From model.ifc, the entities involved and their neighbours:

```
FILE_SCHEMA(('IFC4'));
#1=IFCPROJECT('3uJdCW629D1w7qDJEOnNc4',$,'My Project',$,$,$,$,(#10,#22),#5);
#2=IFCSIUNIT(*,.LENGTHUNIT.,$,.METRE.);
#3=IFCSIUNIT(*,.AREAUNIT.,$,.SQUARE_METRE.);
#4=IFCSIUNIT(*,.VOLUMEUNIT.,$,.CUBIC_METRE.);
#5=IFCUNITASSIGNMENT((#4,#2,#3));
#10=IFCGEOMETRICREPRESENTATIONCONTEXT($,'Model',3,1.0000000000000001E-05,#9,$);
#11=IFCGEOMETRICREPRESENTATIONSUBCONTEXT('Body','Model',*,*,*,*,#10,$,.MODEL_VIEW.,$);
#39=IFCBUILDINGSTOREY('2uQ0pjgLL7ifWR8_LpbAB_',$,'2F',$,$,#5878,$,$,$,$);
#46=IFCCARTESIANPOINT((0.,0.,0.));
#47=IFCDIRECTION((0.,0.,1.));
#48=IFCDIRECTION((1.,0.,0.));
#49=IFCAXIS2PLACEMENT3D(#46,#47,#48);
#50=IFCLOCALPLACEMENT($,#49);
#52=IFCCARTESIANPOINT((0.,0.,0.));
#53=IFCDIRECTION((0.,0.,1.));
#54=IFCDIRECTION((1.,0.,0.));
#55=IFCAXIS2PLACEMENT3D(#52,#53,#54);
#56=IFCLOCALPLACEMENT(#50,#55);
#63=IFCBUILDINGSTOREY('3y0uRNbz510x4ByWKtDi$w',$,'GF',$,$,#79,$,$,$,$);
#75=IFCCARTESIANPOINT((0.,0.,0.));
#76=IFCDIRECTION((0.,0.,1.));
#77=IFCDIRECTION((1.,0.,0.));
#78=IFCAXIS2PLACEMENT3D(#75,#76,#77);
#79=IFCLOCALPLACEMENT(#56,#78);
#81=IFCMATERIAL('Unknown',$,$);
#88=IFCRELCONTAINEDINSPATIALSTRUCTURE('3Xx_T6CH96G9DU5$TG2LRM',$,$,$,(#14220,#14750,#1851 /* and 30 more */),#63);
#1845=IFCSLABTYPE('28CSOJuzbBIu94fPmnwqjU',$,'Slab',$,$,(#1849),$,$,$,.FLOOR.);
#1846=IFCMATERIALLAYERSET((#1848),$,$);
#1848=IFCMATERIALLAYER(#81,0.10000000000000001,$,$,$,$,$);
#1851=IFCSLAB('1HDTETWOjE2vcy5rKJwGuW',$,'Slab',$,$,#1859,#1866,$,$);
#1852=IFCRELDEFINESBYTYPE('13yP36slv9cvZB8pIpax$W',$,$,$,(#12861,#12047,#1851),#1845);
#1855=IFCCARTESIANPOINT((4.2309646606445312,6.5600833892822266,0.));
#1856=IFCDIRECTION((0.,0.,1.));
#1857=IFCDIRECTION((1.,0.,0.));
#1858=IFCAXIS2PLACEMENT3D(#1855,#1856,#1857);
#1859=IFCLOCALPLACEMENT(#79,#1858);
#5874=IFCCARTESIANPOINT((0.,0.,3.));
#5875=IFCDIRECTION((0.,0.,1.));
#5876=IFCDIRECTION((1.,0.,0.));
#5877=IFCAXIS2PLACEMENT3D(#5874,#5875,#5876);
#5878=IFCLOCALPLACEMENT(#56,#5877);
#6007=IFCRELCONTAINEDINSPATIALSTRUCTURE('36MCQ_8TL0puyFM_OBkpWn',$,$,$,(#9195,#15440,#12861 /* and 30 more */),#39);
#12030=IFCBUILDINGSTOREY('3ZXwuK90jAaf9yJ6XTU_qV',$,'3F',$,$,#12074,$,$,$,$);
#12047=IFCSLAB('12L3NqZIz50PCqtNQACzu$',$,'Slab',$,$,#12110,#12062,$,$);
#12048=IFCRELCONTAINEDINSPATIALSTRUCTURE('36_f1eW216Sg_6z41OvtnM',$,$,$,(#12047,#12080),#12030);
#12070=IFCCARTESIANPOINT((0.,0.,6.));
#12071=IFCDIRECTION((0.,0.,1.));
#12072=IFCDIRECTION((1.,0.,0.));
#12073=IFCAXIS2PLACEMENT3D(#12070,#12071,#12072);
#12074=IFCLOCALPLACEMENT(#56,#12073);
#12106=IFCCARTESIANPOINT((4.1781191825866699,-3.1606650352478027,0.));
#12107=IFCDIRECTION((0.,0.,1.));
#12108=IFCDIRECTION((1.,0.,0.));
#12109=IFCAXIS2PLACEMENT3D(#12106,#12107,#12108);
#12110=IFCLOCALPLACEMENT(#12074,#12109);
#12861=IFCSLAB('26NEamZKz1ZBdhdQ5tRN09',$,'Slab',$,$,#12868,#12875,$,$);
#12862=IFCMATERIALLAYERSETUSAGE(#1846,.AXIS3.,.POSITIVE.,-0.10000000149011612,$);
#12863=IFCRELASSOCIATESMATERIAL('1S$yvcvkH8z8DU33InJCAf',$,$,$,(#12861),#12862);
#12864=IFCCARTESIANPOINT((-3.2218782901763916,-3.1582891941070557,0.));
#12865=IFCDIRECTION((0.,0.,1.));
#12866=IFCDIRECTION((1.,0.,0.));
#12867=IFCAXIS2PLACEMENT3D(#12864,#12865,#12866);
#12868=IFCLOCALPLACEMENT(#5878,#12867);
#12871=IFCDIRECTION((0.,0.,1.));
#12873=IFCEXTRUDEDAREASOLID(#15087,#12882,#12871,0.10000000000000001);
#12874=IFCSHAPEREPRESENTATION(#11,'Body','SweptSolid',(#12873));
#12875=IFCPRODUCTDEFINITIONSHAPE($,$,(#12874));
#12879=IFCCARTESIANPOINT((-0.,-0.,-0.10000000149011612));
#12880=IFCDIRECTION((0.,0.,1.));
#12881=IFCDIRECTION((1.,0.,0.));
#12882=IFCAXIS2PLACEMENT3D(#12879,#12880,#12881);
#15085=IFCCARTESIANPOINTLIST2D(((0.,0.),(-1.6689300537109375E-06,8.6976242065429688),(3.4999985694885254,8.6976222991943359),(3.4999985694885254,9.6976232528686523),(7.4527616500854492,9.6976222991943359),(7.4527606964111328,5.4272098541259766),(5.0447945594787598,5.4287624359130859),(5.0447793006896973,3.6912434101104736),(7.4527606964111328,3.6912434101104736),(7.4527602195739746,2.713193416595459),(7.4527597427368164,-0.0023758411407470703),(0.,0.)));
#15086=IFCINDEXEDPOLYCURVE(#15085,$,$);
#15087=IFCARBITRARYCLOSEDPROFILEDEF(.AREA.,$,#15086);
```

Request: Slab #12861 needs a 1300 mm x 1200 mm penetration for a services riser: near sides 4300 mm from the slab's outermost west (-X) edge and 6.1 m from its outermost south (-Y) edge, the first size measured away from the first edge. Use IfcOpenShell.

```python
import numpy as np
import ifcopenshell
import ifcopenshell.api.feature
import ifcopenshell.api.geometry
import ifcopenshell.api.root
import ifcopenshell.geom
import ifcopenshell.util.placement
import ifcopenshell.util.representation
import ifcopenshell.util.shape
import ifcopenshell.util.unit

model = ifcopenshell.open("model.ifc")
unit_scale = ifcopenshell.util.unit.calculate_unit_scale(model)
settings = ifcopenshell.geom.settings()


def volume(element):
    """Net volume in cubic metres, openings subtracted."""
    shape = ifcopenshell.geom.create_shape(settings, element)
    return ifcopenshell.util.shape.get_volume(shape.geometry)


slab = model.by_id(12861)
before = volume(slab)

# Extent in the slab's own axes, in metres. The edges named are its -X and -Y sides.
slab_shape = ifcopenshell.geom.create_shape(settings, slab)
vertices = ifcopenshell.util.shape.get_vertices(slab_shape.geometry)
x_min, y_min, bottom = vertices.min(axis=0)
top = vertices[:, 2].max()

opening = ifcopenshell.api.root.create_entity(model, ifc_class="IfcOpeningElement", name="Services riser opening", predefined_type="OPENING")
context = ifcopenshell.util.representation.get_context(model, "Model", "Body", "MODEL_VIEW")
width, depth = 1.3, 1.2
outline = [(0.0, 0.0), (width, 0.0), (width, depth), (0.0, depth), (0.0, 0.0)]
# Overshoot both faces by 50 mm so the cut is clean.
shape = ifcopenshell.api.geometry.add_slab_representation(
    model, context=context, depth=top - bottom + 0.1, polyline=outline
)
ifcopenshell.api.geometry.assign_representation(model, product=opening, representation=shape)

matrix = ifcopenshell.util.placement.get_local_placement(slab.ObjectPlacement)
matrix[:, 3] = matrix @ np.append(np.array([x_min + 4.3, y_min + 6.1, bottom - 0.05]) / unit_scale, 1.0)
ifcopenshell.api.geometry.edit_object_placement(model, product=opening, matrix=matrix, is_si=False)
ifcopenshell.api.feature.add_feature(model, feature=opening, element=slab)

after = volume(slab)

print(f"slab volume {before:.3f} -> {after:.3f} m3")

model.write("model_edited.ifc")
```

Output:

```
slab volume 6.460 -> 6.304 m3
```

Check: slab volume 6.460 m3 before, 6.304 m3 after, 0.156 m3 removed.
